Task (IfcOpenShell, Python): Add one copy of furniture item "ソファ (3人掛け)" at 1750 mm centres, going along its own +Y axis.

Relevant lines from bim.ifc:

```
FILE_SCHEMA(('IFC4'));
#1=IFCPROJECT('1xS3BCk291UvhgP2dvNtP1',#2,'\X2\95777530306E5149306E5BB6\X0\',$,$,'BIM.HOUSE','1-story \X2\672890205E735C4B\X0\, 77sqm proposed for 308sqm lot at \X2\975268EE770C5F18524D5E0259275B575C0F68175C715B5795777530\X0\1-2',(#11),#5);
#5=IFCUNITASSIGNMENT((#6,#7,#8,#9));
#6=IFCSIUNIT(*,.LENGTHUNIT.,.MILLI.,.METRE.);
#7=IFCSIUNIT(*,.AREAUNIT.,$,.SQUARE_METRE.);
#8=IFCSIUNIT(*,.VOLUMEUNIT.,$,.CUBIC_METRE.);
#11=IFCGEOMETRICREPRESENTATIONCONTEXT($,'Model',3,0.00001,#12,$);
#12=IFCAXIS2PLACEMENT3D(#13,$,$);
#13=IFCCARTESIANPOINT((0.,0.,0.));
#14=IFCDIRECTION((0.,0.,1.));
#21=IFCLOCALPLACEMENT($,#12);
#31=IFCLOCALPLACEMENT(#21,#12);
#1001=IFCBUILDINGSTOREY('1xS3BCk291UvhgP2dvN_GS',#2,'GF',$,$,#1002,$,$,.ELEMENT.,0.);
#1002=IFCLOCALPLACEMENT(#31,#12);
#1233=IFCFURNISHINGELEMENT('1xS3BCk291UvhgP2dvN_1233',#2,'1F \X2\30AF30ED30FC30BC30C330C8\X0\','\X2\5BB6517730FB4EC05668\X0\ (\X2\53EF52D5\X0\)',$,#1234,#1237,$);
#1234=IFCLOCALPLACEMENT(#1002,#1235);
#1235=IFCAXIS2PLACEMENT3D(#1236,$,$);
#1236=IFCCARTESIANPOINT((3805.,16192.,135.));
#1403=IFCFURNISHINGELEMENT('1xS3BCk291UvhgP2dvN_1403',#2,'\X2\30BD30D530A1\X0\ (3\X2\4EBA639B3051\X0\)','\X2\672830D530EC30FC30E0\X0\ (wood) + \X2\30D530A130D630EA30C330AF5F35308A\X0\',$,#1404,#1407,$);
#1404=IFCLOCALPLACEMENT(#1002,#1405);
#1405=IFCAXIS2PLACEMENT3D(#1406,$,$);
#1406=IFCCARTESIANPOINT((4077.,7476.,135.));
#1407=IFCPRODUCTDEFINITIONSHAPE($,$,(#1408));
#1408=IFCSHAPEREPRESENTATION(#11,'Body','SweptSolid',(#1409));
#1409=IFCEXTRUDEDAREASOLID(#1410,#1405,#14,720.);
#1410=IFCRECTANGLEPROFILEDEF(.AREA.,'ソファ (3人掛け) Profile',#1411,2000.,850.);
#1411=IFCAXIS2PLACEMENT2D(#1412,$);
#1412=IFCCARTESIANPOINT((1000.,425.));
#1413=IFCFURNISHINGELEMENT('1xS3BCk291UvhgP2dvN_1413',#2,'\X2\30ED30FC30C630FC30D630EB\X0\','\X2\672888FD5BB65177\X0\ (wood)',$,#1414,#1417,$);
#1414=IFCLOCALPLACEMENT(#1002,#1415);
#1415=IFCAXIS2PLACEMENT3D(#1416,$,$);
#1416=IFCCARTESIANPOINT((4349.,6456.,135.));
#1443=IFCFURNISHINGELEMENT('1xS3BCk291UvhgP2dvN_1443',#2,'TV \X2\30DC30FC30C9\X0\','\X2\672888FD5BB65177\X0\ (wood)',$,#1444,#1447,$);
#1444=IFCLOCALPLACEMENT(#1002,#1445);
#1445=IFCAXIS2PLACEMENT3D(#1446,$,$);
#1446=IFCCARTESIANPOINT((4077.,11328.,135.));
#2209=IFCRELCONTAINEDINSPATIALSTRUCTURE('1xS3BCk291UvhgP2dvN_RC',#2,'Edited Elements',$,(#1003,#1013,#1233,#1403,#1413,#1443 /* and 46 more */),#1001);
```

```python
import ifcopenshell
import ifcopenshell.api.geometry
import ifcopenshell.api.root
import ifcopenshell.util.element
import ifcopenshell.util.placement
import ifcopenshell.util.unit

model = ifcopenshell.open("bim.ifc")
unit_scale = ifcopenshell.util.unit.calculate_unit_scale(model)


def reuse_history(source, copy):
    """copy_class also copies each property set's owner history, people and application; keep the originals."""
    for rel in copy.IsDefinedBy:
        if rel.is_a("IfcRelDefinesByProperties") and (history := rel.RelatingPropertyDefinition.OwnerHistory):
            rel.RelatingPropertyDefinition.OwnerHistory = source.OwnerHistory
            ifcopenshell.util.element.remove_deep2(model, history)


source = model.by_guid("1xS3BCk291UvhgP2dvN_1403")
base = ifcopenshell.util.placement.get_local_placement(source.ObjectPlacement)
step = base[:3, 1] * 1.75 / unit_scale

for i in range(1, 2):
    copy = ifcopenshell.api.root.copy_class(model, product=source)
    copy.Representation = ifcopenshell.util.element.copy_deep(
        model, source.Representation, exclude=["IfcGeometricRepresentationContext", "IfcRepresentationMap"]
    )
    reuse_history(source, copy)
    matrix = base.copy()
    matrix[:3, 3] += i * step
    print("added at", matrix[:3, 3].round(3) + 0.0)
    ifcopenshell.api.geometry.edit_object_placement(model, product=copy, matrix=matrix, is_si=False)

model.write("bim-out.ifc")
```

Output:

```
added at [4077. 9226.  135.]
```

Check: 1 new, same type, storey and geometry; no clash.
